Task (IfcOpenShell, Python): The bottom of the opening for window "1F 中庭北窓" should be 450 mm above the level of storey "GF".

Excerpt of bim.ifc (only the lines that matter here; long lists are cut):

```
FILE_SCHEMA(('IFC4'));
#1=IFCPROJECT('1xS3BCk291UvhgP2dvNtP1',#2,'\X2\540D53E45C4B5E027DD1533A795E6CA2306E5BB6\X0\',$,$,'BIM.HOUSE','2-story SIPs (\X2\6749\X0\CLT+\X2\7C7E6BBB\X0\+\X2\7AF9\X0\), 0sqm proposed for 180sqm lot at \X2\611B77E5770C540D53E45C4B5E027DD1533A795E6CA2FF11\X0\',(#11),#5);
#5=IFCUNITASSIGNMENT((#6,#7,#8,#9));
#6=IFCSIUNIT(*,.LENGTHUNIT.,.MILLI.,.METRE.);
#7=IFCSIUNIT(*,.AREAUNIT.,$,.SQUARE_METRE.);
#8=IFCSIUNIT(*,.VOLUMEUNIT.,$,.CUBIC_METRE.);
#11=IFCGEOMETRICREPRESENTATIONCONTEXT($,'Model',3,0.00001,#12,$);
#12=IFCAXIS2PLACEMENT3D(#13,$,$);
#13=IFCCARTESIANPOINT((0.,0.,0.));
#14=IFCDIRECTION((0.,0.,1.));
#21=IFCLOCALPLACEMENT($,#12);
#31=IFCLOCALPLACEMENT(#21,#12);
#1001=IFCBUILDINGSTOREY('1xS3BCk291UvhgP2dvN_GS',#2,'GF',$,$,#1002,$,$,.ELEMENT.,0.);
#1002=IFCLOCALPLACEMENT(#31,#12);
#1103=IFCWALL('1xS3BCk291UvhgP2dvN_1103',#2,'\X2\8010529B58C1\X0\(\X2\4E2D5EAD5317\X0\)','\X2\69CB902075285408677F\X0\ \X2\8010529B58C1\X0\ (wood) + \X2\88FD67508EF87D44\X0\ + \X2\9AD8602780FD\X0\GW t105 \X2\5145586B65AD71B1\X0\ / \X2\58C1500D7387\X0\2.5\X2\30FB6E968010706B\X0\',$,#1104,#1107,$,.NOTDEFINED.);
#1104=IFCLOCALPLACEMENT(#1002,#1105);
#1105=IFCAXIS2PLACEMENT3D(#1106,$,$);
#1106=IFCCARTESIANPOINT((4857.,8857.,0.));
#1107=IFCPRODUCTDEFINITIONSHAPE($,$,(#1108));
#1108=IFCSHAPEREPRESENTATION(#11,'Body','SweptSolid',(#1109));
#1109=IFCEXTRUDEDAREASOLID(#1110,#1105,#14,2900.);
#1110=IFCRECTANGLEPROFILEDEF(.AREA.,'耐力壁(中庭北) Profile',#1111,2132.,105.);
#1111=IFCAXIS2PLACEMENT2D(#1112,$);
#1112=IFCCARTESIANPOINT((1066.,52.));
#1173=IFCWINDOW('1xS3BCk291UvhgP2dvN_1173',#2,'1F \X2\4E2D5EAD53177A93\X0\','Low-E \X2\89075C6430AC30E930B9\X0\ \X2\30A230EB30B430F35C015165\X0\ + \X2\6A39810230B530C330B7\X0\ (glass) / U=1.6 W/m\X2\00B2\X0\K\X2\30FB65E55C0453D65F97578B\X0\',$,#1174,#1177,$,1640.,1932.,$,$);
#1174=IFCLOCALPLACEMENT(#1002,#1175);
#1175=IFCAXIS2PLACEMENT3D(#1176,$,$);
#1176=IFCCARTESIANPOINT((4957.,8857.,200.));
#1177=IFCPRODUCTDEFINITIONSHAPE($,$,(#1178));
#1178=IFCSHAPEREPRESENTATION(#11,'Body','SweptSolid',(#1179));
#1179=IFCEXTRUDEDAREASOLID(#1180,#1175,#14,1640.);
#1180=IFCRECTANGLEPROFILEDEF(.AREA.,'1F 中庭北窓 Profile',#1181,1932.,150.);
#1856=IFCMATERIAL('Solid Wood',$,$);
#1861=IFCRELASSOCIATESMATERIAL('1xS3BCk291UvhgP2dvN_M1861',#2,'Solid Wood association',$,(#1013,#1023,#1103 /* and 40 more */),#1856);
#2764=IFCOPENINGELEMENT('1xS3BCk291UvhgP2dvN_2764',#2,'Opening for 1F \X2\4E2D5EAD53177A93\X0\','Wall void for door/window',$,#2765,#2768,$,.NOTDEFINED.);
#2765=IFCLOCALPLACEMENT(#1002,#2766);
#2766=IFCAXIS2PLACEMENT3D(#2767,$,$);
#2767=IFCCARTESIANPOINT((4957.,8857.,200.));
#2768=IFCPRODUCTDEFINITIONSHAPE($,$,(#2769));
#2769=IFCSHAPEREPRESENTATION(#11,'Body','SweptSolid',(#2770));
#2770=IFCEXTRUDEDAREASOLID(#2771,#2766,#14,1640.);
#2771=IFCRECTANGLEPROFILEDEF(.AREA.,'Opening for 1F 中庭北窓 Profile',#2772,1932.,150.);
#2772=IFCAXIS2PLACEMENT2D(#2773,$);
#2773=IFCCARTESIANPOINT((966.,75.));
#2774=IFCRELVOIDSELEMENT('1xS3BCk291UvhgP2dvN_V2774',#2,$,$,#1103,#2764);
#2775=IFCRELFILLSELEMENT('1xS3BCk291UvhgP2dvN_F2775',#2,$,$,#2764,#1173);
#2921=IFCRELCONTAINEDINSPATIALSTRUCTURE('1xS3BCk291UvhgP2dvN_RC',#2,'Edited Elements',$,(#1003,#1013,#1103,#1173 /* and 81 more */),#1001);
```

```python
import numpy as np
import ifcopenshell
import ifcopenshell.api.geometry
import ifcopenshell.geom
import ifcopenshell.util.element
import ifcopenshell.util.placement
import ifcopenshell.util.shape
import ifcopenshell.util.unit

model = ifcopenshell.open("bim.ifc")
unit_scale = ifcopenshell.util.unit.calculate_unit_scale(model)

window = model.by_id(1173)
opening = window.FillsVoids[0].RelatingOpeningElement
storey = ifcopenshell.util.element.get_container(window, ifc_class="IfcBuildingStorey")
level = ifcopenshell.util.placement.get_local_placement(storey.ObjectPlacement)[2, 3]

# The opening's origin need not be at the sill, so measure its lowest point.
shape = ifcopenshell.geom.create_shape(ifcopenshell.geom.settings(), opening)
bottom = ifcopenshell.util.shape.get_shape_bottom_elevation(shape, shape.geometry) / unit_scale
dz = level + 0.45 / unit_scale - bottom

shift = np.array([0.0, 0.0, dz])
# The window is not placed relative to its opening, so move both.
for product in (opening, window):
    matrix = ifcopenshell.util.placement.get_local_placement(product.ObjectPlacement)
    matrix[:3, 3] += shift
    ifcopenshell.api.geometry.edit_object_placement(model, product=product, matrix=matrix, is_si=False)

print(f"moved by {dz * unit_scale:+.3f} m")

model.write("bim_rev.ifc")
```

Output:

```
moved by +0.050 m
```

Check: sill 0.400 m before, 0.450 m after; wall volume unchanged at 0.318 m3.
